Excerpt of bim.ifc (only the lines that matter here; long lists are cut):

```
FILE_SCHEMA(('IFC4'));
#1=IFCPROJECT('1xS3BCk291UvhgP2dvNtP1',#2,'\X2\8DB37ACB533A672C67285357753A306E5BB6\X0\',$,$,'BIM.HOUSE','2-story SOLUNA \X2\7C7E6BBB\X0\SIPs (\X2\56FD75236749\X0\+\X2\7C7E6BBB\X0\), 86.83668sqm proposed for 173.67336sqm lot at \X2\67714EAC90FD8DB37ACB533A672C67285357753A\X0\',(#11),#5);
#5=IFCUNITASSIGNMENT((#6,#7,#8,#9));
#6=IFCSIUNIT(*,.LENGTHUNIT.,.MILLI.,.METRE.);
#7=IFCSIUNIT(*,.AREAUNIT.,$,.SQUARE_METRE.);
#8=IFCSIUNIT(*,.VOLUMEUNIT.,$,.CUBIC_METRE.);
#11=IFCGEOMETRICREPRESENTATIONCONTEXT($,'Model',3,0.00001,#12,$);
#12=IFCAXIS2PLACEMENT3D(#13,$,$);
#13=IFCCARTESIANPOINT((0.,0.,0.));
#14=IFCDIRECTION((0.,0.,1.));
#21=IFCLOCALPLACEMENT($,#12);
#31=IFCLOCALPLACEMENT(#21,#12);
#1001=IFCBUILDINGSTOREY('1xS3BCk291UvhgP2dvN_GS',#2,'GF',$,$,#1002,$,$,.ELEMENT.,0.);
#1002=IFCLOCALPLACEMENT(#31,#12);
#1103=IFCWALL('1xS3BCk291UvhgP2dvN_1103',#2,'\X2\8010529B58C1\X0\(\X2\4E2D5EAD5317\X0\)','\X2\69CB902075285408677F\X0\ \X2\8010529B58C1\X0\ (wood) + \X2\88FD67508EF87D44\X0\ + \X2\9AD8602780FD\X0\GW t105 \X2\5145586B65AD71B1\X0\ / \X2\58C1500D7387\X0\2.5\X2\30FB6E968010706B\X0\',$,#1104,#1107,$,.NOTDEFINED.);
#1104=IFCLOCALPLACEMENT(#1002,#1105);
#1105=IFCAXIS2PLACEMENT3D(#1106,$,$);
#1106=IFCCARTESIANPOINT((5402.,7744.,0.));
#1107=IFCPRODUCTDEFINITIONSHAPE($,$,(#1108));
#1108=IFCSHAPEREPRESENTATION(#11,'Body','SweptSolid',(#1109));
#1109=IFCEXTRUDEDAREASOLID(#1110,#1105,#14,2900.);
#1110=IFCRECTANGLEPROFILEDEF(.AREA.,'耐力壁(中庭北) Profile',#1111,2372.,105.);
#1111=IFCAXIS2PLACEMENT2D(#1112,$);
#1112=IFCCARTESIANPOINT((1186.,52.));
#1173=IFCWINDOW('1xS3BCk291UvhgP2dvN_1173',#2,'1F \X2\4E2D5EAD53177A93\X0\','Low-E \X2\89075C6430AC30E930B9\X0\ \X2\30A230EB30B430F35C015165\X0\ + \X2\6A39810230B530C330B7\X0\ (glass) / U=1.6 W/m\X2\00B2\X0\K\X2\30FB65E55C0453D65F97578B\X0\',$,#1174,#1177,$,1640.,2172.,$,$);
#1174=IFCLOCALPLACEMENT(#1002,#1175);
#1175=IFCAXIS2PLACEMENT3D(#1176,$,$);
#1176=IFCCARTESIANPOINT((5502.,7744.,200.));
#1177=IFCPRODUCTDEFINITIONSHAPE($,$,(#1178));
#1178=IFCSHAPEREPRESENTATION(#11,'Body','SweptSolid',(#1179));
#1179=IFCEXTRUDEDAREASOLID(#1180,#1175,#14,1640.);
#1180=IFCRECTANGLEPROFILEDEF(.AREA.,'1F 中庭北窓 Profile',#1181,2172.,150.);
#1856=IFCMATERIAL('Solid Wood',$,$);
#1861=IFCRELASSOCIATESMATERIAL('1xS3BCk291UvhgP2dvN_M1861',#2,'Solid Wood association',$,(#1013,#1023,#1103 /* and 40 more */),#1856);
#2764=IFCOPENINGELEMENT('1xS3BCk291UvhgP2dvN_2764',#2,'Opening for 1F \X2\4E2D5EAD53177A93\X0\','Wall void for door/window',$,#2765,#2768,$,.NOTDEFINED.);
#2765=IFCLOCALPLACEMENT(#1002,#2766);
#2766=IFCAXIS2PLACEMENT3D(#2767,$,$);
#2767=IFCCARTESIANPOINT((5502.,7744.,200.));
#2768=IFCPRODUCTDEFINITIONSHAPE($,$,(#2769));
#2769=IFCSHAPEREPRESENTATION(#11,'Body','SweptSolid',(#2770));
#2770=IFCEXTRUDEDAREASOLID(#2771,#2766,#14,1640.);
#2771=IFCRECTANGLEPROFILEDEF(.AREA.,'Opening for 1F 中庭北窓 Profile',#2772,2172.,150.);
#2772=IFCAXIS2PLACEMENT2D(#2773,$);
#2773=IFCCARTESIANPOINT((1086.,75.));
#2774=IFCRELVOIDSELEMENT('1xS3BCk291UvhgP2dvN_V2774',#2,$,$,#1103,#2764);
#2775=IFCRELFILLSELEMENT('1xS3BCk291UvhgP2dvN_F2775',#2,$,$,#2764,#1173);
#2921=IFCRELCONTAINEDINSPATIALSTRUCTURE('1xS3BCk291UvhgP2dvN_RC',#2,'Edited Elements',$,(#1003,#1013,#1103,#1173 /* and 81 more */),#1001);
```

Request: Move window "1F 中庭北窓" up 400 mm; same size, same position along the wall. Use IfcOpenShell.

```python
import numpy as np
import ifcopenshell
import ifcopenshell.api.geometry
import ifcopenshell.util.placement
import ifcopenshell.util.unit

model = ifcopenshell.open("bim.ifc")
unit_scale = ifcopenshell.util.unit.calculate_unit_scale(model)

window = model.by_guid("1xS3BCk291UvhgP2dvN_1173")
opening = window.FillsVoids[0].RelatingOpeningElement
dz = 400.0

shift = np.array([0.0, 0.0, dz])
# The window is not placed relative to its opening, so move both.
for product in (opening, window):
    matrix = ifcopenshell.util.placement.get_local_placement(product.ObjectPlacement)
    matrix[:3, 3] += shift
    ifcopenshell.api.geometry.edit_object_placement(model, product=product, matrix=matrix, is_si=False)

print(f"moved by {dz * unit_scale:+.3f} m")

model.write("bim_updated.ifc")
```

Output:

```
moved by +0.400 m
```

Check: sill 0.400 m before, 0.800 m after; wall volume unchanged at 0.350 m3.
